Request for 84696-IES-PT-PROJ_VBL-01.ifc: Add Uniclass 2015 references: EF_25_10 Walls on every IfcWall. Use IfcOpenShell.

First a look at what the model holds.

```python
import ifcopenshell

model = ifcopenshell.open("84696-IES-PT-PROJ_VBL-01.ifc")
print(model.schema)
print("classifications:", [c.Name for c in model.by_type("IfcClassification")])
for ifc_class in ("IfcDoor", "IfcRoof", "IfcStair", "IfcWall", "IfcWindow"):
    print(ifc_class, len(model.by_type(ifc_class)))
```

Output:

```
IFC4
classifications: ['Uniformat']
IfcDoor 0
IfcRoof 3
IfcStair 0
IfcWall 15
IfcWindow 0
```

```python
import ifcopenshell
import ifcopenshell.api.classification

model = ifcopenshell.open("84696-IES-PT-PROJ_VBL-01.ifc")

system = ifcopenshell.api.classification.add_classification(model, classification="Uniclass 2015")

codes = {
    "IfcWall": ("EF_25_10", "Walls"),
}
for ifc_class, (code, name) in codes.items():
    products = model.by_type(ifc_class)
    ifcopenshell.api.classification.add_reference(
        model, products=products, classification=system, identification=code, name=name
    )
    print(code, len(products))

model.write("84696-IES-PT-PROJ_VBL-01-out.ifc")
```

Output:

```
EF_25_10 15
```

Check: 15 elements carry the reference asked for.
